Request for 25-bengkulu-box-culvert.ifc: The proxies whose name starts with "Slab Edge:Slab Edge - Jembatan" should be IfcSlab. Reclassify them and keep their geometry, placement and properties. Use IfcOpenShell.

First a look at what the model holds.

```python
import re

import ifcopenshell

model = ifcopenshell.open("25-bengkulu-box-culvert.ifc")
print(model.schema)
seen = {}
for e in model.by_type("IfcBuildingElementProxy"):
    name = re.sub(r":\d+(:\d+)?$", "", e.Name or "")  # drop the element id that some exporters append
    seen[name] = seen.get(name, 0) + 1
for name, count in sorted(seen.items()):
    print(count, "x", name)
```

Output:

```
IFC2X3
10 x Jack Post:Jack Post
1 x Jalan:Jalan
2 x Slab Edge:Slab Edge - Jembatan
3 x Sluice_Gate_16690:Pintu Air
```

```python
import ifcopenshell
import ifcopenshell.api.root

model = ifcopenshell.open("25-bengkulu-box-culvert.ifc")

proxies = [e.id() for e in model.by_type("IfcBuildingElementProxy") if (e.Name or "").startswith("Slab Edge:Slab Edge - Jembatan")]
for step_id in proxies:
    proxy = model.by_id(step_id)
    # Reclassifying a typed element also reclassifies its type and the type's other occurrences.
    if proxy.is_a("IfcBuildingElementProxy"):
        ifcopenshell.api.root.reassign_class(model, product=proxy, ifc_class="IfcSlab", predefined_type="FLOOR")

print(sum(model.by_id(i).is_a("IfcSlab") for i in proxies), "reclassified")

model.write("25-bengkulu-box-culvert_updated.ifc")
```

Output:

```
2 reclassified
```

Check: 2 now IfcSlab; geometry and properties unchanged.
